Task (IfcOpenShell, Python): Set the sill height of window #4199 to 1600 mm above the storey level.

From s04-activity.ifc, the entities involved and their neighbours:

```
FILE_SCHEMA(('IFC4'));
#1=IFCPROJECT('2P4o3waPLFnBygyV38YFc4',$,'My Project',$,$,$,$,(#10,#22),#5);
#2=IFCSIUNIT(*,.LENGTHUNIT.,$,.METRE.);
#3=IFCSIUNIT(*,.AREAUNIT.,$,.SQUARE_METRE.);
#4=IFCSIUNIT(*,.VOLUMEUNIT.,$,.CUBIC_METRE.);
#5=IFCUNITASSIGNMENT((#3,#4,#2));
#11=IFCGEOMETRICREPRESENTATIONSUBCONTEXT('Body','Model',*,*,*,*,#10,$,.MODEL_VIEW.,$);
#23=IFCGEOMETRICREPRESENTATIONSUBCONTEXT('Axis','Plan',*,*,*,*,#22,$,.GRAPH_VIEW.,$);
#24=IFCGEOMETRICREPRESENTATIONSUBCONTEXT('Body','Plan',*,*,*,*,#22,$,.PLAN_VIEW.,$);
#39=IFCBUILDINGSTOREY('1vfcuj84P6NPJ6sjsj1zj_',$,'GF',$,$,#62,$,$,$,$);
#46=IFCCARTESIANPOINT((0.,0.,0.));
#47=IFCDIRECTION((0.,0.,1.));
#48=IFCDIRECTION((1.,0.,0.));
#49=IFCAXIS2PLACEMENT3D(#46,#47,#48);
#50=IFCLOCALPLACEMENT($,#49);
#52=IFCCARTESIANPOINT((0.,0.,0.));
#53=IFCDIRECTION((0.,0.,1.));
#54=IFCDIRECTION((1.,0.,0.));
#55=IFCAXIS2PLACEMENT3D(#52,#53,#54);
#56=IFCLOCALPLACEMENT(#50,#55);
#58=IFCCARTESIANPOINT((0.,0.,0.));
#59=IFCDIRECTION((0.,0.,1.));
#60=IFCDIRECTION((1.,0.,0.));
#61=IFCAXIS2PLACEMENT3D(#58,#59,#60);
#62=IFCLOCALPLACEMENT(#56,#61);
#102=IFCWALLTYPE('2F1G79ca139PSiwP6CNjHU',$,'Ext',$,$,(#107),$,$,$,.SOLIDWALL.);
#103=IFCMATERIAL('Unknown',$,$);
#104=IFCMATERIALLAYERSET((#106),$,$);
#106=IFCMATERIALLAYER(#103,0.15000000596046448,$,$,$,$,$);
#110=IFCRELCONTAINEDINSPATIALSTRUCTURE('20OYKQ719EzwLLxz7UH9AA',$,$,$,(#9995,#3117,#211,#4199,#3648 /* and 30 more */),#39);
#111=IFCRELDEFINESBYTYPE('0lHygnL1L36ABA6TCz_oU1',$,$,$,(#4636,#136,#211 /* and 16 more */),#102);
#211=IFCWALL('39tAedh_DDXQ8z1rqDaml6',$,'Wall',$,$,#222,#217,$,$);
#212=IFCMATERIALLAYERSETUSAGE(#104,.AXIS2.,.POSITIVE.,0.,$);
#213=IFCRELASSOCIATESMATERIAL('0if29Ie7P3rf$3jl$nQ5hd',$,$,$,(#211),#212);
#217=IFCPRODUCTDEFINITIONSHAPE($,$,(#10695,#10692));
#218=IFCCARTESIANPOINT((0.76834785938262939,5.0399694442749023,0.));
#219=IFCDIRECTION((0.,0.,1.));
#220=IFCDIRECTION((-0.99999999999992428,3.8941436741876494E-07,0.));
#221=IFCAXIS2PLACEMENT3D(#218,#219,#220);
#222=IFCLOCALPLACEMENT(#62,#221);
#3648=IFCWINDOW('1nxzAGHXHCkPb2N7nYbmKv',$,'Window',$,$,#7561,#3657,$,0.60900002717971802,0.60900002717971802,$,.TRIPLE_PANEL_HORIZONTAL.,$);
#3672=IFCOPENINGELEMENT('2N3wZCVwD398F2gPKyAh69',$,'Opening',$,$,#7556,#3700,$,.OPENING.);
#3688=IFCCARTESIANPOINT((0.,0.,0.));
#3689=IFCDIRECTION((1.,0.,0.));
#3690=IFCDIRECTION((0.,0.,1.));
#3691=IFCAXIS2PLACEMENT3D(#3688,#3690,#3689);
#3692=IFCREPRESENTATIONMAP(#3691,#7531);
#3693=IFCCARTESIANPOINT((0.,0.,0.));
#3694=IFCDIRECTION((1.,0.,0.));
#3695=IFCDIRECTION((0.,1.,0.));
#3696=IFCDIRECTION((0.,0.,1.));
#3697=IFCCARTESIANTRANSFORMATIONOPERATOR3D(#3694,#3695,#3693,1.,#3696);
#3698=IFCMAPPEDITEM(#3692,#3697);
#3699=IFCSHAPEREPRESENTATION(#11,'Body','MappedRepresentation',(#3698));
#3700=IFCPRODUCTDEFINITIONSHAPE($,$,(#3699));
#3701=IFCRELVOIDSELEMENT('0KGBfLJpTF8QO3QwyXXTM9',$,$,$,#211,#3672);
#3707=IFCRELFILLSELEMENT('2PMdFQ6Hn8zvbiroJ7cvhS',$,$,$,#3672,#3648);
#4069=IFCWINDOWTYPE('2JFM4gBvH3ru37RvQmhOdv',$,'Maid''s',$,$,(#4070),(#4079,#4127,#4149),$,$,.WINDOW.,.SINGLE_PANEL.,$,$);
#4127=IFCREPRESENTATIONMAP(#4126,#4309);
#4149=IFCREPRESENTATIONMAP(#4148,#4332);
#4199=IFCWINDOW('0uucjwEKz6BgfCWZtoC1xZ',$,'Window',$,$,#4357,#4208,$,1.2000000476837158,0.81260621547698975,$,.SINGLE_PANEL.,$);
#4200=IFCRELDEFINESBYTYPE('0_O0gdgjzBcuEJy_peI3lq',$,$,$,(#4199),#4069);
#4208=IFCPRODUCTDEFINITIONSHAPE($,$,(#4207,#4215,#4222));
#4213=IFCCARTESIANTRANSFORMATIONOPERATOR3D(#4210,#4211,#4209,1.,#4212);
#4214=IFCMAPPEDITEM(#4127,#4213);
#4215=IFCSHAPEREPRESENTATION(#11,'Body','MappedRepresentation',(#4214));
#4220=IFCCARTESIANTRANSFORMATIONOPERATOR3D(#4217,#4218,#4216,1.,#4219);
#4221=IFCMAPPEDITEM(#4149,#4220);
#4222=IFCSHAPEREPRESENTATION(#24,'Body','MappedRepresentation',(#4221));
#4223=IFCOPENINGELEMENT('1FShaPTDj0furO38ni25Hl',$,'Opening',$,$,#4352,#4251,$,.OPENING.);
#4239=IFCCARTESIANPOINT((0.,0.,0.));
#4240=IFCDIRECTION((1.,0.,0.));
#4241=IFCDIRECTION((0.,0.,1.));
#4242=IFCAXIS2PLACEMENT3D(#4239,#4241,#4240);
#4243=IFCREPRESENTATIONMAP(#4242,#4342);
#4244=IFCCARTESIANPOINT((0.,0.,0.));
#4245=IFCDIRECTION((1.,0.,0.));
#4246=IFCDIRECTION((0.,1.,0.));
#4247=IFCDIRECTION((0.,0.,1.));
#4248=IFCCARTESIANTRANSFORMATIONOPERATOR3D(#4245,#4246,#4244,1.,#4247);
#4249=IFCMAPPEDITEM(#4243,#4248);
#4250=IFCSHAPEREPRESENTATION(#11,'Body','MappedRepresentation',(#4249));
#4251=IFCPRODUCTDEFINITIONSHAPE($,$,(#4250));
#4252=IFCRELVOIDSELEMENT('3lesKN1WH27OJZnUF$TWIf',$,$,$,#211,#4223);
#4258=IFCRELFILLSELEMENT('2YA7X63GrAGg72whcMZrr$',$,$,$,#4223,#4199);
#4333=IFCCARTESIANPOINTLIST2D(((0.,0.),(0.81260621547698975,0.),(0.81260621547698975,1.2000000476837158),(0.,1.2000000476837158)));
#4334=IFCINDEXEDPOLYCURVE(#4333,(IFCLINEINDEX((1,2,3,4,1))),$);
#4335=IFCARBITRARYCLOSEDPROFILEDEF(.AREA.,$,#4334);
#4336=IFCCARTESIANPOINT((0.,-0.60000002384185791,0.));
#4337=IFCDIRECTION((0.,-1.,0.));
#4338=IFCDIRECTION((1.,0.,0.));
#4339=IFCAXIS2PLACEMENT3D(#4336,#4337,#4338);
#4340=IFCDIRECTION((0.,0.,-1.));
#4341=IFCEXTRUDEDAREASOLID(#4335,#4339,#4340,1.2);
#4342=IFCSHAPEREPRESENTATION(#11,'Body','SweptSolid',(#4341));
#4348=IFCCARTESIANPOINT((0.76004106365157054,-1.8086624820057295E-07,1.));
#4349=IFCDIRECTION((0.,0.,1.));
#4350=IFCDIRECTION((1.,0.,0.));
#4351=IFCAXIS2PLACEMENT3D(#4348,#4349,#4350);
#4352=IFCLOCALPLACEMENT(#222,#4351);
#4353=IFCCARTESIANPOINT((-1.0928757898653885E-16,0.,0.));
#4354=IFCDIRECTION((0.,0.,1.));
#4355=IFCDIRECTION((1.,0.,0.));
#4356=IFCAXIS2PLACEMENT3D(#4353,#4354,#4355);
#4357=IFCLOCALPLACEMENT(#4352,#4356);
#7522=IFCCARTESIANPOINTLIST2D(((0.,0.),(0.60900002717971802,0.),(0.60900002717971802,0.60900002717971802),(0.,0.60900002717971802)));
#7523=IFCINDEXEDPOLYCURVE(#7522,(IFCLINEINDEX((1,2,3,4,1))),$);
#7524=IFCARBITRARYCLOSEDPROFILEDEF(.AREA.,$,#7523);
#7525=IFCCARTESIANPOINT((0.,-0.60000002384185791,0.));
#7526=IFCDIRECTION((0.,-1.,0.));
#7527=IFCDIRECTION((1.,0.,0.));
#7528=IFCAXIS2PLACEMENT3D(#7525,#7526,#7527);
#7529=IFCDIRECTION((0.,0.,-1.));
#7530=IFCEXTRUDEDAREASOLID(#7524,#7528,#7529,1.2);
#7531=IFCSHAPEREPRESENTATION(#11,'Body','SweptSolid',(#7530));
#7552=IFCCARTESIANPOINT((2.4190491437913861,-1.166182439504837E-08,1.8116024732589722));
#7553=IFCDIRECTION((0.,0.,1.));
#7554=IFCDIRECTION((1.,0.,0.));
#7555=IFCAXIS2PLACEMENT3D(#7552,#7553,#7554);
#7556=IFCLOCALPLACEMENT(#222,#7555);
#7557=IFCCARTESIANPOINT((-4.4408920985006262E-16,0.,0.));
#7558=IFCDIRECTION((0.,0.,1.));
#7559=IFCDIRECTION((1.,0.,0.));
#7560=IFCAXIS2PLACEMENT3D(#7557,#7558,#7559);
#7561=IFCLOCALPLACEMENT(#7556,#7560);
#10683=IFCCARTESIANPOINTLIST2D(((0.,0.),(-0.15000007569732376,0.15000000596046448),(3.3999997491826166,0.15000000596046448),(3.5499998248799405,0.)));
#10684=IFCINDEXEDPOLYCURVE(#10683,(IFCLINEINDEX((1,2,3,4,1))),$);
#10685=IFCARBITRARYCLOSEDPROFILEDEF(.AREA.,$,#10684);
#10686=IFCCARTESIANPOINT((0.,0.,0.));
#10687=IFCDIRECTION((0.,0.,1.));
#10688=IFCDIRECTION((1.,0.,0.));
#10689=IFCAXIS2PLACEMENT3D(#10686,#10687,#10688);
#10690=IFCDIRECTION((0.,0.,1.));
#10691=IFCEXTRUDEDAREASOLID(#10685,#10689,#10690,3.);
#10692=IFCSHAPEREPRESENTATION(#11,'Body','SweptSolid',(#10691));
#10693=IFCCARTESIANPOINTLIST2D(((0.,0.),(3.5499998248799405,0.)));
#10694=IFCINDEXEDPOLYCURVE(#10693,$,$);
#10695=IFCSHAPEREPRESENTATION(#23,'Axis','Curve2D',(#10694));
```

```python
import numpy as np
import ifcopenshell
import ifcopenshell.api.geometry
import ifcopenshell.geom
import ifcopenshell.util.element
import ifcopenshell.util.placement
import ifcopenshell.util.shape
import ifcopenshell.util.unit

model = ifcopenshell.open("s04-activity.ifc")
unit_scale = ifcopenshell.util.unit.calculate_unit_scale(model)

window = model.by_guid("0uucjwEKz6BgfCWZtoC1xZ")
opening = window.FillsVoids[0].RelatingOpeningElement
storey = ifcopenshell.util.element.get_container(window, ifc_class="IfcBuildingStorey")
level = ifcopenshell.util.placement.get_local_placement(storey.ObjectPlacement)[2, 3]

# The opening's origin need not be at the sill, so measure its lowest point.
shape = ifcopenshell.geom.create_shape(ifcopenshell.geom.settings(), opening)
bottom = ifcopenshell.util.shape.get_shape_bottom_elevation(shape, shape.geometry) / unit_scale
dz = level + 1.6 / unit_scale - bottom

shift = np.array([0.0, 0.0, dz])
# The window is placed relative to its opening, so it follows when the opening moves.
matrix = ifcopenshell.util.placement.get_local_placement(opening.ObjectPlacement)
matrix[:3, 3] += shift
ifcopenshell.api.geometry.edit_object_placement(
    model, product=opening, matrix=matrix, is_si=False, should_transform_children=True
)

print(f"moved by {dz * unit_scale:+.3f} m")

model.write("s04-activity-out.ifc")
```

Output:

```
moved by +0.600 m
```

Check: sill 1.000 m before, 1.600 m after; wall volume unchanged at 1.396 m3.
